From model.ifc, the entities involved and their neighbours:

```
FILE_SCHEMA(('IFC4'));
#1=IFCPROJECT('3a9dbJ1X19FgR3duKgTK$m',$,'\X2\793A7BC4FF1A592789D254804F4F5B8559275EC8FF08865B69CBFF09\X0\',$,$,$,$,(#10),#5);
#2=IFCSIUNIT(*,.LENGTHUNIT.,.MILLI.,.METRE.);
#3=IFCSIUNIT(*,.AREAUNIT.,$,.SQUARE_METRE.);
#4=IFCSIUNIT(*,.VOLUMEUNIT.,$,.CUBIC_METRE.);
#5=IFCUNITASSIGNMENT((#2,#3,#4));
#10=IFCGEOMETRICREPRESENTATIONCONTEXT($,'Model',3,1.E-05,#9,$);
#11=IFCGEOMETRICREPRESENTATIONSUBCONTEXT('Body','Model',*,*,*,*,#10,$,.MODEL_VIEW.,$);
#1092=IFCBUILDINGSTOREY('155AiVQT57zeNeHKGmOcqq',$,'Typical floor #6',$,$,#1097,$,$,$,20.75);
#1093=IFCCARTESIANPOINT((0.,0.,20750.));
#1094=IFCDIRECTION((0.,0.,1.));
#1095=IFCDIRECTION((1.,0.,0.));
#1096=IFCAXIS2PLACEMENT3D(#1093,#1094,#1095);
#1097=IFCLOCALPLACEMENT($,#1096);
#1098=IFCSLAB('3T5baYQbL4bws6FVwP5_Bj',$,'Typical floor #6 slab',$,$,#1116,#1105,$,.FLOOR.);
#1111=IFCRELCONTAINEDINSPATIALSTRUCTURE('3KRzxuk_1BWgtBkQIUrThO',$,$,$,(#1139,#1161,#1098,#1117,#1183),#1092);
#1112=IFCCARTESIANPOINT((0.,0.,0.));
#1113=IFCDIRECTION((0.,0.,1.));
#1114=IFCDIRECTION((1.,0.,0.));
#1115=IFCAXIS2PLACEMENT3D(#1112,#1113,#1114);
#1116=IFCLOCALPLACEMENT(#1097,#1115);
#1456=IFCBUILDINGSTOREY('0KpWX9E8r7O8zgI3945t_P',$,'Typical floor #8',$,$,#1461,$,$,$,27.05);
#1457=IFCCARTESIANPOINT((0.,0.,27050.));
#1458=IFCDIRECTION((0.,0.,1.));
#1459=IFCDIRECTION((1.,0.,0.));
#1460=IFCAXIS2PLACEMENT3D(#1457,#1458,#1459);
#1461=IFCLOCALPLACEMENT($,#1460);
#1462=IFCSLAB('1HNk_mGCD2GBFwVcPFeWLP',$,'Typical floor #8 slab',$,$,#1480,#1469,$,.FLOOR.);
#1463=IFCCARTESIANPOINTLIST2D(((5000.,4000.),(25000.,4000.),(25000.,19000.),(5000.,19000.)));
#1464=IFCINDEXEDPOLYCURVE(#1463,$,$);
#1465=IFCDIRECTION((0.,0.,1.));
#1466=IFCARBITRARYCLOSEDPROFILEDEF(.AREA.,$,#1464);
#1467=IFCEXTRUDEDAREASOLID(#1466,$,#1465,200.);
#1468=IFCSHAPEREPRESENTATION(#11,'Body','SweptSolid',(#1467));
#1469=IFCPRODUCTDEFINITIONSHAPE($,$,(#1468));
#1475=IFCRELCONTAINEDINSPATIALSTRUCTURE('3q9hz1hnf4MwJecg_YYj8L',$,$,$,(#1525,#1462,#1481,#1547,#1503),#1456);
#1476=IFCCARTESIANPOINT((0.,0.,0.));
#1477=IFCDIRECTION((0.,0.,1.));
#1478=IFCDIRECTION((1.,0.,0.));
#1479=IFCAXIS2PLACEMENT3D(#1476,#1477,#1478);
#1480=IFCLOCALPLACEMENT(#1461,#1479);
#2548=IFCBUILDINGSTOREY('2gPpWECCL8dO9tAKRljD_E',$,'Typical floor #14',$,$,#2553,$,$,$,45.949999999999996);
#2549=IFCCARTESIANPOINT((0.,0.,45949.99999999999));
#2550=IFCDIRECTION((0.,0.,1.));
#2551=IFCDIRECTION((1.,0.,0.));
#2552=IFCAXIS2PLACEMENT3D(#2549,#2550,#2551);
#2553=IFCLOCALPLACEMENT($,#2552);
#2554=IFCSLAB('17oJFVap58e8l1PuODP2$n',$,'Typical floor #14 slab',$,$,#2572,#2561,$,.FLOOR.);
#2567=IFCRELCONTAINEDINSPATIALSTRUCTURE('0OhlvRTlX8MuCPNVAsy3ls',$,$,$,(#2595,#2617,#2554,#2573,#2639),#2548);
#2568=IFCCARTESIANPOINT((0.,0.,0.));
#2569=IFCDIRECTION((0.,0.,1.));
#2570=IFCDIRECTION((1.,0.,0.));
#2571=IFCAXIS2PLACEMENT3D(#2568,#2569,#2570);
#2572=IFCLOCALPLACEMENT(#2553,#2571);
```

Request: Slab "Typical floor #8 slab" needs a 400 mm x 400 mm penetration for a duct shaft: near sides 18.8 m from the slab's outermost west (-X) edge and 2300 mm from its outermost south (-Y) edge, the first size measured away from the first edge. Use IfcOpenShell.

```python
import numpy as np
import ifcopenshell
import ifcopenshell.api.feature
import ifcopenshell.api.geometry
import ifcopenshell.api.root
import ifcopenshell.geom
import ifcopenshell.util.placement
import ifcopenshell.util.representation
import ifcopenshell.util.shape
import ifcopenshell.util.unit

model = ifcopenshell.open("model.ifc")
unit_scale = ifcopenshell.util.unit.calculate_unit_scale(model)
settings = ifcopenshell.geom.settings()


def volume(element):
    """Net volume in cubic metres, openings subtracted."""
    shape = ifcopenshell.geom.create_shape(settings, element)
    return ifcopenshell.util.shape.get_volume(shape.geometry)


slab = model.by_id(1462)
before = volume(slab)

# Extent in the slab's own axes, in metres. The edges named are its -X and -Y sides.
slab_shape = ifcopenshell.geom.create_shape(settings, slab)
vertices = ifcopenshell.util.shape.get_vertices(slab_shape.geometry)
x_min, y_min, bottom = vertices.min(axis=0)
top = vertices[:, 2].max()

opening = ifcopenshell.api.root.create_entity(model, ifc_class="IfcOpeningElement", name="Duct shaft opening", predefined_type="OPENING")
context = ifcopenshell.util.representation.get_context(model, "Model", "Body", "MODEL_VIEW")
width, depth = 0.4, 0.4
outline = [(0.0, 0.0), (width, 0.0), (width, depth), (0.0, depth), (0.0, 0.0)]
# Overshoot both faces by 50 mm so the cut is clean.
shape = ifcopenshell.api.geometry.add_slab_representation(
    model, context=context, depth=top - bottom + 0.1, polyline=outline
)
ifcopenshell.api.geometry.assign_representation(model, product=opening, representation=shape)

matrix = ifcopenshell.util.placement.get_local_placement(slab.ObjectPlacement)
matrix[:, 3] = matrix @ np.append(np.array([x_min + 18.8, y_min + 2.3, bottom - 0.05]) / unit_scale, 1.0)
ifcopenshell.api.geometry.edit_object_placement(model, product=opening, matrix=matrix, is_si=False)
ifcopenshell.api.feature.add_feature(model, feature=opening, element=slab)

after = volume(slab)

print(f"slab volume {before:.3f} -> {after:.3f} m3")

model.write("model_updated.ifc")
```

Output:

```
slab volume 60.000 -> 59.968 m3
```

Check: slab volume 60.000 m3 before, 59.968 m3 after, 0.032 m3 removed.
